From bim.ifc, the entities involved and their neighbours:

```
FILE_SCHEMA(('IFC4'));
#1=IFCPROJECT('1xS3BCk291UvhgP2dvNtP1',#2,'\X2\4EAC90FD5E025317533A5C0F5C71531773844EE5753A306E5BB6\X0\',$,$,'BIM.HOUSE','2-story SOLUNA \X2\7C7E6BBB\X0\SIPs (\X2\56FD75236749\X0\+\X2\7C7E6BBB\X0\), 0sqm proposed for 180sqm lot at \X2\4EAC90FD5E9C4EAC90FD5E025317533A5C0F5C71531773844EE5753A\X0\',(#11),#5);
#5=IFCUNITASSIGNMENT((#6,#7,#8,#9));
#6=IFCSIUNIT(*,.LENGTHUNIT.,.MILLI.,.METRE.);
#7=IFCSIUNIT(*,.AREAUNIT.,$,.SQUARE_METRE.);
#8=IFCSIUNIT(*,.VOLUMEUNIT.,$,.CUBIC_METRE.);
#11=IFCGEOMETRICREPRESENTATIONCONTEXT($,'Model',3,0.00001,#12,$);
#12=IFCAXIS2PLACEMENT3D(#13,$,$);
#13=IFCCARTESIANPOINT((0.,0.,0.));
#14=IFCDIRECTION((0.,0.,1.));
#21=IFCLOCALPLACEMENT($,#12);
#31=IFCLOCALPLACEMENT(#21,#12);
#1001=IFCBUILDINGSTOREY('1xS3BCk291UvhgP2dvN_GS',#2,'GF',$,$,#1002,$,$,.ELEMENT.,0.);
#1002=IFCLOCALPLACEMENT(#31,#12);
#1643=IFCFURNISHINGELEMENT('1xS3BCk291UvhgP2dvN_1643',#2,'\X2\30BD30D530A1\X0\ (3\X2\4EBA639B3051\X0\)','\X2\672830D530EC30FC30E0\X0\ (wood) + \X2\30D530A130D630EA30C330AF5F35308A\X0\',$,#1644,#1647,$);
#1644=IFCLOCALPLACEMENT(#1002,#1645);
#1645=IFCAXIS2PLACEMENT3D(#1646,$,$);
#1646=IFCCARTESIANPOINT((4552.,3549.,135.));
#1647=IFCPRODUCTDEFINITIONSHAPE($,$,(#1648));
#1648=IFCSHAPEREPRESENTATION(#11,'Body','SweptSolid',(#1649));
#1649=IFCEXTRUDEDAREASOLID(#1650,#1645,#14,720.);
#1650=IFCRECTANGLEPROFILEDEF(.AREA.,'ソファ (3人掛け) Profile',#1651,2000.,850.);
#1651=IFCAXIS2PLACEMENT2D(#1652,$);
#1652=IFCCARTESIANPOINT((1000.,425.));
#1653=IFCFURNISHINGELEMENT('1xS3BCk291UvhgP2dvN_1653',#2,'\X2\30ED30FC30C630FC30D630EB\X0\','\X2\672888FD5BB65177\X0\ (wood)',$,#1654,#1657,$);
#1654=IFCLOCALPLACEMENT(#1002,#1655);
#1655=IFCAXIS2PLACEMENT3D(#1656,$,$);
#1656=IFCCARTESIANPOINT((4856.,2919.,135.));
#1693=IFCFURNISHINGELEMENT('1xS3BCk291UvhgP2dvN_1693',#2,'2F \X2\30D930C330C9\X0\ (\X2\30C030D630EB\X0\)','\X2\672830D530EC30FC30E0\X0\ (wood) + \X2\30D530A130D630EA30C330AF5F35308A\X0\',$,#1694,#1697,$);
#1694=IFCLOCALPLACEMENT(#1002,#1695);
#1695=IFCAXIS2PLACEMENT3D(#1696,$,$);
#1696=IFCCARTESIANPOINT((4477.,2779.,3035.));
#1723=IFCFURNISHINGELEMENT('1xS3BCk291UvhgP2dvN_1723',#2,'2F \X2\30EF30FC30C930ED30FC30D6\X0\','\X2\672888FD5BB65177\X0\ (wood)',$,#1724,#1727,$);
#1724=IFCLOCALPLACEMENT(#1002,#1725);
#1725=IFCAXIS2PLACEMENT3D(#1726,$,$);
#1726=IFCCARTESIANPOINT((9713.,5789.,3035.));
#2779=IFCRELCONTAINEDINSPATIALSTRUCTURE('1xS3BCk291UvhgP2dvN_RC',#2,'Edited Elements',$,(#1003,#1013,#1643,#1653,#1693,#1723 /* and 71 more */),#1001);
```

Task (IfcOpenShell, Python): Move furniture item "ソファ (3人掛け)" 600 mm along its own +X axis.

```python
import ifcopenshell
import ifcopenshell.api.geometry
import ifcopenshell.util.placement

model = ifcopenshell.open("bim.ifc")

item = model.by_id(1643)
matrix = ifcopenshell.util.placement.get_local_placement(item.ObjectPlacement)
matrix[:3, 3] += matrix[:3, 0] * 600.0
ifcopenshell.api.geometry.edit_object_placement(model, product=item, matrix=matrix, is_si=False)

print(ifcopenshell.util.placement.get_local_placement(item.ObjectPlacement).round(3) + 0.0)

model.write("bim-out.ifc")
```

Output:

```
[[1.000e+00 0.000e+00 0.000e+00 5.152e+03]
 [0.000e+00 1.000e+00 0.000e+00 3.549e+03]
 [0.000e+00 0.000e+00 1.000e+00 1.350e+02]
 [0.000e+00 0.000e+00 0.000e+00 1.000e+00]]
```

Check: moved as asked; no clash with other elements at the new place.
